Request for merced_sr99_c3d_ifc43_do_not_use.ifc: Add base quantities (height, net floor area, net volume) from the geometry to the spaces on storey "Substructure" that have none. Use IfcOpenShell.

First a look at what the model holds.

```python
import ifcopenshell
import ifcopenshell.util.element
import ifcopenshell.util.unit

model = ifcopenshell.open("merced_sr99_c3d_ifc43_do_not_use.ifc")
print(model.schema)
for unit_type in ("LENGTHUNIT", "AREAUNIT", "VOLUMEUNIT"):
    print(unit_type, ifcopenshell.util.unit.calculate_unit_scale(model, unit_type))
storey = next(s for s in model.by_type("IfcBuildingStorey") if s.Name == "Substructure")
spaces = [e for e in ifcopenshell.util.element.get_decomposition(storey) if e.is_a("IfcSpace")]
for e in sorted(spaces, key=lambda e: e.id()):
    print(e.id(), e.is_a(), e.Name, list(ifcopenshell.util.element.get_psets(e, qtos_only=True)), sep=" | ")
```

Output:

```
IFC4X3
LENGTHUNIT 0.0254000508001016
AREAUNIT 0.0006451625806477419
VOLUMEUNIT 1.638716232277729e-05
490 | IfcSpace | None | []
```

```python
import ifcopenshell
import ifcopenshell.api.pset
import ifcopenshell.geom
import ifcopenshell.util.element
import ifcopenshell.util.shape
import ifcopenshell.util.unit

model = ifcopenshell.open("merced_sr99_c3d_ifc43_do_not_use.ifc")
unit_scale = ifcopenshell.util.unit.calculate_unit_scale(model)
area_scale = ifcopenshell.util.unit.calculate_unit_scale(model, "AREAUNIT")
volume_scale = ifcopenshell.util.unit.calculate_unit_scale(model, "VOLUMEUNIT")
settings = ifcopenshell.geom.settings()

storey = next(s for s in model.by_type("IfcBuildingStorey") if s.Name == "Substructure")
spaces = [e for e in ifcopenshell.util.element.get_decomposition(storey) if e.is_a("IfcSpace")]

for e in sorted(spaces, key=lambda e: e.id()):
    if ifcopenshell.util.element.get_psets(e, qtos_only=True, should_inherit=False):
        continue
    # Geometry comes back in metres, in the element's own axes.
    shape = ifcopenshell.geom.create_shape(settings, e)
    values = {
        "Height": ifcopenshell.util.shape.get_z(shape.geometry) / unit_scale,
        "NetFloorArea": ifcopenshell.util.shape.get_footprint_area(shape.geometry) / area_scale,
        "NetVolume": ifcopenshell.util.shape.get_volume(shape.geometry) / volume_scale,
    }
    qto = ifcopenshell.api.pset.add_qto(model, product=e, name="Qto_SpaceBaseQuantities")
    ifcopenshell.api.pset.edit_qto(model, qto=qto, properties=values)
    print(e.id(), {k: round(v, 3) for k, v in values.items()})

model.write("merced_sr99_c3d_ifc43_do_not_use-out.ifc")
```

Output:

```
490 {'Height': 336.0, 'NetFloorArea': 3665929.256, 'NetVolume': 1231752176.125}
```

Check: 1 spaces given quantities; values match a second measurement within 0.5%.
